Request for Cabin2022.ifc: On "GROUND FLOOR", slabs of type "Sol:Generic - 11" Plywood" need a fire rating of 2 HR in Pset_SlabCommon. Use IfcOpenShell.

First a look at what the model holds.

```python
import ifcopenshell
import ifcopenshell.util.element

model = ifcopenshell.open("Cabin2022.ifc")
print(model.schema)
storey = next(s for s in model.by_type("IfcBuildingStorey") if s.Name == "GROUND FLOOR")
slabs = [e for e in ifcopenshell.util.element.get_decomposition(storey) if e.is_a("IfcSlab")]
seen = {}
for e in slabs:
    element_type = ifcopenshell.util.element.get_type(e)
    key = (element_type.Name if element_type != e and element_type else None, ifcopenshell.util.element.get_pset(e, "Pset_SlabCommon", "FireRating"))
    seen[key] = seen.get(key, 0) + 1
for (name, value), count in sorted(seen.items(), key=str):
    print(count, "x", name, "|", value)
```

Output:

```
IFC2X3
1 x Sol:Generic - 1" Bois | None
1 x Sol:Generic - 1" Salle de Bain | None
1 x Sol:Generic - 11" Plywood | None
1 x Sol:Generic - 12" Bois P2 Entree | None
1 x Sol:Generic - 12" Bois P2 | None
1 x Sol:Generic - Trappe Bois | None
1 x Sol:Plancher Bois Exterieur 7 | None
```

```python
import ifcopenshell
import ifcopenshell.api.pset
import ifcopenshell.util.element

model = ifcopenshell.open("Cabin2022.ifc")

storey = next(s for s in model.by_type("IfcBuildingStorey") if s.Name == "GROUND FLOOR")
slabs = [e for e in ifcopenshell.util.element.get_decomposition(storey) if e.is_a("IfcSlab")]

count = 0
for e in slabs:
    element_type = ifcopenshell.util.element.get_type(e)
    if element_type in (None, e) or element_type.Name != 'Sol:Generic - 11" Plywood':
        continue
    # add_pset returns the element's existing set when there is one.
    pset = ifcopenshell.api.pset.add_pset(model, product=e, name="Pset_SlabCommon")
    ifcopenshell.api.pset.edit_pset(model, pset=pset, properties={"FireRating": "2 HR"})
    count += 1

print(count, "slabs updated")

model.write("Cabin2022_rev.ifc")
```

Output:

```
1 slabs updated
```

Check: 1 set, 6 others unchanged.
